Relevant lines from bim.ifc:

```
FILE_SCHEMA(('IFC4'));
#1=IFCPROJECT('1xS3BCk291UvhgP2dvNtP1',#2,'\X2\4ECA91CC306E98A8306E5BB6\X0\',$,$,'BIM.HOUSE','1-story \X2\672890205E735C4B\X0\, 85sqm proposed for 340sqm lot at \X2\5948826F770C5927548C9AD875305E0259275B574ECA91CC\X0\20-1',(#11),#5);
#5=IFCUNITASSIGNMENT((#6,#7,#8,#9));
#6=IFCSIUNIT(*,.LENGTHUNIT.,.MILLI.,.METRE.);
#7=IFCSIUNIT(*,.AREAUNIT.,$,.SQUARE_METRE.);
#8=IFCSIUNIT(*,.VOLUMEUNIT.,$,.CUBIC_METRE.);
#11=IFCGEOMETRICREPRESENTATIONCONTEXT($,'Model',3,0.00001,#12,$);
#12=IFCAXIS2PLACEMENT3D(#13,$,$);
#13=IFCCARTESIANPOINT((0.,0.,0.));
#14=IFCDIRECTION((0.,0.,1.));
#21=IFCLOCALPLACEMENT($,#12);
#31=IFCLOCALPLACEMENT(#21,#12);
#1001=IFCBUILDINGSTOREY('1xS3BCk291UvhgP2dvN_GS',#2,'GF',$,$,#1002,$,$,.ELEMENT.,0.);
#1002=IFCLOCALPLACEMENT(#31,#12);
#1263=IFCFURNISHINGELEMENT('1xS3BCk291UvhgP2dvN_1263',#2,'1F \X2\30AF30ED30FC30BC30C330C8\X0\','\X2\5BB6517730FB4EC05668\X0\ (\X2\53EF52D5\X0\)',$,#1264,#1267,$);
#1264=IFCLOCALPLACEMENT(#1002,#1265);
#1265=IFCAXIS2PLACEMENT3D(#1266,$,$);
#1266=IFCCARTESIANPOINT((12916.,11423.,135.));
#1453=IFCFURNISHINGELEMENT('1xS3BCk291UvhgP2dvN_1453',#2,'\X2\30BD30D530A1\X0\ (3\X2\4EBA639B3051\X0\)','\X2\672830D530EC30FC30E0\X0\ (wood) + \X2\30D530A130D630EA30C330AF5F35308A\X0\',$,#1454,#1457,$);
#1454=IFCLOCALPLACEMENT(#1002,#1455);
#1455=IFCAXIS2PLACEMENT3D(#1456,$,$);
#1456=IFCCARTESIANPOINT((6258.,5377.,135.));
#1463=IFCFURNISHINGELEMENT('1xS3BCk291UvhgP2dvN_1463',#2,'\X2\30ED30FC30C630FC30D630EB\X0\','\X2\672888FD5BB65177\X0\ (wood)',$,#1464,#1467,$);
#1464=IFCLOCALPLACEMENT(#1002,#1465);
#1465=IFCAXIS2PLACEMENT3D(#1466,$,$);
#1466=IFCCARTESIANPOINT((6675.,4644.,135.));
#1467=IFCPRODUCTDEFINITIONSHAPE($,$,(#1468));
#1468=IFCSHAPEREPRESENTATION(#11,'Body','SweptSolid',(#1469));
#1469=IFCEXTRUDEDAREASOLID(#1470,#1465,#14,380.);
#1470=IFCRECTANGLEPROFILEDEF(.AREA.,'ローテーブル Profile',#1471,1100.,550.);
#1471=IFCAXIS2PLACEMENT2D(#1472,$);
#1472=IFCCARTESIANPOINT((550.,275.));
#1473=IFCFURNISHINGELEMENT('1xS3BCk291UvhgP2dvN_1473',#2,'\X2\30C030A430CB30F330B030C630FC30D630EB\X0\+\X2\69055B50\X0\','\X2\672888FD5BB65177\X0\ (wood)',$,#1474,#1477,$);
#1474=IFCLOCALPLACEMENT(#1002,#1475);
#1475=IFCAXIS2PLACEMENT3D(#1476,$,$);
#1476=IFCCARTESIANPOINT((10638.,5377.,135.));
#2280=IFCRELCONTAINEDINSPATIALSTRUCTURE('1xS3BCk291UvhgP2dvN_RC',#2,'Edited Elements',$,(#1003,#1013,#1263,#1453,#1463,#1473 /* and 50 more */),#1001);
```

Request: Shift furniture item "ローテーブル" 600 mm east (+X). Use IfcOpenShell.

```python
import ifcopenshell
import ifcopenshell.api.geometry
import ifcopenshell.util.placement

model = ifcopenshell.open("bim.ifc")

item = model.by_id(1463)
matrix = ifcopenshell.util.placement.get_local_placement(item.ObjectPlacement)
matrix[0, 3] += 600.0
ifcopenshell.api.geometry.edit_object_placement(model, product=item, matrix=matrix, is_si=False)

print(ifcopenshell.util.placement.get_local_placement(item.ObjectPlacement).round(3) + 0.0)

model.write("bim_updated.ifc")
```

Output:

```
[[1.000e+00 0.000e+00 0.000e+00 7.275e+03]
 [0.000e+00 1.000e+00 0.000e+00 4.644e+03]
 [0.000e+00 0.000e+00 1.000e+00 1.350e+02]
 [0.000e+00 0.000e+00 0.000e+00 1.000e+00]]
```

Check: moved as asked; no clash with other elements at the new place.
